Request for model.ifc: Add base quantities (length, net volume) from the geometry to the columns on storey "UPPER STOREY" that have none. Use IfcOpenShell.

First a look at what the model holds.

```python
import ifcopenshell
import ifcopenshell.util.element
import ifcopenshell.util.unit

model = ifcopenshell.open("model.ifc")
print(model.schema)
for unit_type in ("LENGTHUNIT", "AREAUNIT", "VOLUMEUNIT"):
    print(unit_type, ifcopenshell.util.unit.calculate_unit_scale(model, unit_type))
storey = next(s for s in model.by_type("IfcBuildingStorey") if s.Name == "UPPER STOREY")
columns = [e for e in ifcopenshell.util.element.get_decomposition(storey) if e.is_a("IfcColumn")]
for e in sorted(columns, key=lambda e: e.id()):
    print(e.id(), e.is_a(), e.Name, list(ifcopenshell.util.element.get_psets(e, qtos_only=True)), sep=" | ")
```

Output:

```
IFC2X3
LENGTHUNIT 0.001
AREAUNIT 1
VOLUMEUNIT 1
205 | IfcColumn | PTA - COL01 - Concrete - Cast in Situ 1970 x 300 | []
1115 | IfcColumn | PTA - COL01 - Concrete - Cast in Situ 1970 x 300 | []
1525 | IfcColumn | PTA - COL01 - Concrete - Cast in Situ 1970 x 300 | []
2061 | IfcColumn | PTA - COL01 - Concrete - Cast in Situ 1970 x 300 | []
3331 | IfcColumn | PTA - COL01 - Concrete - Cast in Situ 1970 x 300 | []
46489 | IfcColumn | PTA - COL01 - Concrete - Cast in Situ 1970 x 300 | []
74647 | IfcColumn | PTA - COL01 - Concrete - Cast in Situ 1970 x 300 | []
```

```python
import ifcopenshell
import ifcopenshell.api.pset
import ifcopenshell.geom
import ifcopenshell.util.element
import ifcopenshell.util.shape
import ifcopenshell.util.unit

model = ifcopenshell.open("model.ifc")
unit_scale = ifcopenshell.util.unit.calculate_unit_scale(model)
volume_scale = ifcopenshell.util.unit.calculate_unit_scale(model, "VOLUMEUNIT")
settings = ifcopenshell.geom.settings()

storey = next(s for s in model.by_type("IfcBuildingStorey") if s.Name == "UPPER STOREY")
columns = [e for e in ifcopenshell.util.element.get_decomposition(storey) if e.is_a("IfcColumn")]

for e in sorted(columns, key=lambda e: e.id()):
    if ifcopenshell.util.element.get_psets(e, qtos_only=True, should_inherit=False):
        continue
    # Geometry comes back in metres, in the element's own axes.
    shape = ifcopenshell.geom.create_shape(settings, e)
    values = {
        "Length": ifcopenshell.util.shape.get_z(shape.geometry) / unit_scale,
        "NetVolume": ifcopenshell.util.shape.get_volume(shape.geometry) / volume_scale,
    }
    qto = ifcopenshell.api.pset.add_qto(model, product=e, name="BaseQuantities")
    ifcopenshell.api.pset.edit_qto(model, qto=qto, properties=values)
    print(e.id(), {k: round(v, 3) for k, v in values.items()})

model.write("model_v2.ifc")
```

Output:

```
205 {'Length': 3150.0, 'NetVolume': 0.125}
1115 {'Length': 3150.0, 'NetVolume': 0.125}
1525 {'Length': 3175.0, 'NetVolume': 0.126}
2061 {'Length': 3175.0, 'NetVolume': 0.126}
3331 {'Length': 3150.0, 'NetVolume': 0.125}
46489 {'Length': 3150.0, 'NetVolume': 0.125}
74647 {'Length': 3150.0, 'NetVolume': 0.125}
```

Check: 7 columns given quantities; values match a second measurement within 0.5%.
